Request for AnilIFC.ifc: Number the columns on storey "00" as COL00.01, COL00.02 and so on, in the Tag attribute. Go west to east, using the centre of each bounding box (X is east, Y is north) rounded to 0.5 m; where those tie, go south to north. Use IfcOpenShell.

First a look at what the model holds.

```python
import ifcopenshell
import ifcopenshell.util.element
import ifcopenshell.util.placement

model = ifcopenshell.open("AnilIFC.ifc")
print(model.schema)
storey = next(s for s in model.by_type("IfcBuildingStorey") if s.Name == "00")
columns = [e for e in ifcopenshell.util.element.get_decomposition(storey) if e.is_a("IfcColumn")]
for e in sorted(columns, key=lambda e: e.id()):
    origin = ifcopenshell.util.placement.get_local_placement(e.ObjectPlacement)[:3, 3]
    print(e.id(), e.Tag, e.Name, origin.round(2) + 0.0, sep=" | ")
```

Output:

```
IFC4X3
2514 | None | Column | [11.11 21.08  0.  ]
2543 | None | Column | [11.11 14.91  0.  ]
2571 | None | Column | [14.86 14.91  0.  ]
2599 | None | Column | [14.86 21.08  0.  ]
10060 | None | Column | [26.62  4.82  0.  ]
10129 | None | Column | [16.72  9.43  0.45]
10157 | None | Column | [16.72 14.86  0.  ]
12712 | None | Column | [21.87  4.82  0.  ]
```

```python
import ifcopenshell
import ifcopenshell.geom
import ifcopenshell.util.element
import ifcopenshell.util.shape

model = ifcopenshell.open("AnilIFC.ifc")
settings = ifcopenshell.geom.settings()
settings.set("use-world-coords", True)


def centre(element):
    shape = ifcopenshell.geom.create_shape(settings, element)
    return ifcopenshell.util.shape.get_bbox_centroid(shape.geometry)


storey = next(s for s in model.by_type("IfcBuildingStorey") if s.Name == "00")
columns = [e for e in ifcopenshell.util.element.get_decomposition(storey) if e.is_a("IfcColumn")]

# Insertion points can sit at a corner or the storey origin, so sort by the geometry (in metres).
centres = {e: centre(e) for e in columns}
columns.sort(key=lambda e: (round(centres[e][0] / 0.5), centres[e][1]))

for i, e in enumerate(columns, start=1):
    number = f"COL00.{i:02d}"
    e.Tag = number
    print(e.id(), number)

model.write("AnilIFC_rev.ifc")
```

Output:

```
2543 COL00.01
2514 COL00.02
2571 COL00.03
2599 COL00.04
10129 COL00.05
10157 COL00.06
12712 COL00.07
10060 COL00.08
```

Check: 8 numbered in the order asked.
